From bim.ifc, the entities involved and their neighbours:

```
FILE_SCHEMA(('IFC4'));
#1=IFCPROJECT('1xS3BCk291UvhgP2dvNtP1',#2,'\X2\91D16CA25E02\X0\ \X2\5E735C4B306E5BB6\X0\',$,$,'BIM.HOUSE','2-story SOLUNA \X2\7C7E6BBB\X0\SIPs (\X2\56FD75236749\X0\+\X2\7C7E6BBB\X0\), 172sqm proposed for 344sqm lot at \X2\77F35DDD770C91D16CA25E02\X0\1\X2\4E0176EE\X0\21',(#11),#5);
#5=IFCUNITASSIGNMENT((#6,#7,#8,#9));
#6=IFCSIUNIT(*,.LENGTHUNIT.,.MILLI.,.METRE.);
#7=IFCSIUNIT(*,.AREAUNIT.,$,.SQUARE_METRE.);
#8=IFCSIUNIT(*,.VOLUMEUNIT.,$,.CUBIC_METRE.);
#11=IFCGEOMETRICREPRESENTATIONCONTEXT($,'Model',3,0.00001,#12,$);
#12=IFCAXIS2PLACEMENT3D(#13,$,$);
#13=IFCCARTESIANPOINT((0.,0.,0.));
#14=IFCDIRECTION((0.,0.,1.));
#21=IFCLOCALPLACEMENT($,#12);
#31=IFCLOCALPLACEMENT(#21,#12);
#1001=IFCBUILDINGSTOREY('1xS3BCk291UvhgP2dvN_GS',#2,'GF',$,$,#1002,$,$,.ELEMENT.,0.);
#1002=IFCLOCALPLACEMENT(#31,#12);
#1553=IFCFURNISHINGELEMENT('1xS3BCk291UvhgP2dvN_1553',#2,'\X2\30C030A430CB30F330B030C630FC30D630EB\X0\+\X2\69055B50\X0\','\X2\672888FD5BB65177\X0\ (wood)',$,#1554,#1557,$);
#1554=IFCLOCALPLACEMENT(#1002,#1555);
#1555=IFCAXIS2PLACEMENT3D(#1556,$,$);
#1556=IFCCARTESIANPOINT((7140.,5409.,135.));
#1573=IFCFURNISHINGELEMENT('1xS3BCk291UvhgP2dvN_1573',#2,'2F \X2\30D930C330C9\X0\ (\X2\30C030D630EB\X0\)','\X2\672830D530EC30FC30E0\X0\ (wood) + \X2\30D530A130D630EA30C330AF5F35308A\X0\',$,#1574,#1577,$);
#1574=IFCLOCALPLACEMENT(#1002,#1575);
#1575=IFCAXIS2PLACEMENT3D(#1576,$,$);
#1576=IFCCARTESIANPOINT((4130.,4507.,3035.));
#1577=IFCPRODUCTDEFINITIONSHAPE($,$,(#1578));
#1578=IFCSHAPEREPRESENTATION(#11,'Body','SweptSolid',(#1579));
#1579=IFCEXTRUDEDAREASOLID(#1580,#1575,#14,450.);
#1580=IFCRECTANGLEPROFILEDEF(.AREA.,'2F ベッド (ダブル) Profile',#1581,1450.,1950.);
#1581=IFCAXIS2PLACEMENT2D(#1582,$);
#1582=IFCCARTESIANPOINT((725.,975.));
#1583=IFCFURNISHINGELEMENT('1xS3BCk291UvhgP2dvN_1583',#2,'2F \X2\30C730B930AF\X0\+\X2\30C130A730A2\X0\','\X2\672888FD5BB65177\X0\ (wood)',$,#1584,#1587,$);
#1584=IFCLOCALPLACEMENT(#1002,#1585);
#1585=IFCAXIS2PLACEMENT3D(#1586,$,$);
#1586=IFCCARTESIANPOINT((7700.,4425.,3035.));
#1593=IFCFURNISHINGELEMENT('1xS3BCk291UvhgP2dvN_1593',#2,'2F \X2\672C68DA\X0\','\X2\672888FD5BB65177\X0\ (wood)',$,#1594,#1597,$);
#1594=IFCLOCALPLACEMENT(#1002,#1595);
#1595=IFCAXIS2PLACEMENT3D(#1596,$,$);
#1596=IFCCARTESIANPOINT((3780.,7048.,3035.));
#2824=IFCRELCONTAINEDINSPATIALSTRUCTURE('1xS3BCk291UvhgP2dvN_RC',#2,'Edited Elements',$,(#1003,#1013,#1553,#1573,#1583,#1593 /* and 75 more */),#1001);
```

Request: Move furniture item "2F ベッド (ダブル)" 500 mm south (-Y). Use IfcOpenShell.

```python
import ifcopenshell
import ifcopenshell.api.geometry
import ifcopenshell.util.placement
import ifcopenshell.util.unit

model = ifcopenshell.open("bim.ifc")
unit_scale = ifcopenshell.util.unit.calculate_unit_scale(model)

item = model.by_guid("1xS3BCk291UvhgP2dvN_1573")
matrix = ifcopenshell.util.placement.get_local_placement(item.ObjectPlacement)
matrix[1, 3] -= 0.5 / unit_scale
ifcopenshell.api.geometry.edit_object_placement(model, product=item, matrix=matrix, is_si=False)

print(ifcopenshell.util.placement.get_local_placement(item.ObjectPlacement).round(3) + 0.0)

model.write("bim_edited.ifc")
```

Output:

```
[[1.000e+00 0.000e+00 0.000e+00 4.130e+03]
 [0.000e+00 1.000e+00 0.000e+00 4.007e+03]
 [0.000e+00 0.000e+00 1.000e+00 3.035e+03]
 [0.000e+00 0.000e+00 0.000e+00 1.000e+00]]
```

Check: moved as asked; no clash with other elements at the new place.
